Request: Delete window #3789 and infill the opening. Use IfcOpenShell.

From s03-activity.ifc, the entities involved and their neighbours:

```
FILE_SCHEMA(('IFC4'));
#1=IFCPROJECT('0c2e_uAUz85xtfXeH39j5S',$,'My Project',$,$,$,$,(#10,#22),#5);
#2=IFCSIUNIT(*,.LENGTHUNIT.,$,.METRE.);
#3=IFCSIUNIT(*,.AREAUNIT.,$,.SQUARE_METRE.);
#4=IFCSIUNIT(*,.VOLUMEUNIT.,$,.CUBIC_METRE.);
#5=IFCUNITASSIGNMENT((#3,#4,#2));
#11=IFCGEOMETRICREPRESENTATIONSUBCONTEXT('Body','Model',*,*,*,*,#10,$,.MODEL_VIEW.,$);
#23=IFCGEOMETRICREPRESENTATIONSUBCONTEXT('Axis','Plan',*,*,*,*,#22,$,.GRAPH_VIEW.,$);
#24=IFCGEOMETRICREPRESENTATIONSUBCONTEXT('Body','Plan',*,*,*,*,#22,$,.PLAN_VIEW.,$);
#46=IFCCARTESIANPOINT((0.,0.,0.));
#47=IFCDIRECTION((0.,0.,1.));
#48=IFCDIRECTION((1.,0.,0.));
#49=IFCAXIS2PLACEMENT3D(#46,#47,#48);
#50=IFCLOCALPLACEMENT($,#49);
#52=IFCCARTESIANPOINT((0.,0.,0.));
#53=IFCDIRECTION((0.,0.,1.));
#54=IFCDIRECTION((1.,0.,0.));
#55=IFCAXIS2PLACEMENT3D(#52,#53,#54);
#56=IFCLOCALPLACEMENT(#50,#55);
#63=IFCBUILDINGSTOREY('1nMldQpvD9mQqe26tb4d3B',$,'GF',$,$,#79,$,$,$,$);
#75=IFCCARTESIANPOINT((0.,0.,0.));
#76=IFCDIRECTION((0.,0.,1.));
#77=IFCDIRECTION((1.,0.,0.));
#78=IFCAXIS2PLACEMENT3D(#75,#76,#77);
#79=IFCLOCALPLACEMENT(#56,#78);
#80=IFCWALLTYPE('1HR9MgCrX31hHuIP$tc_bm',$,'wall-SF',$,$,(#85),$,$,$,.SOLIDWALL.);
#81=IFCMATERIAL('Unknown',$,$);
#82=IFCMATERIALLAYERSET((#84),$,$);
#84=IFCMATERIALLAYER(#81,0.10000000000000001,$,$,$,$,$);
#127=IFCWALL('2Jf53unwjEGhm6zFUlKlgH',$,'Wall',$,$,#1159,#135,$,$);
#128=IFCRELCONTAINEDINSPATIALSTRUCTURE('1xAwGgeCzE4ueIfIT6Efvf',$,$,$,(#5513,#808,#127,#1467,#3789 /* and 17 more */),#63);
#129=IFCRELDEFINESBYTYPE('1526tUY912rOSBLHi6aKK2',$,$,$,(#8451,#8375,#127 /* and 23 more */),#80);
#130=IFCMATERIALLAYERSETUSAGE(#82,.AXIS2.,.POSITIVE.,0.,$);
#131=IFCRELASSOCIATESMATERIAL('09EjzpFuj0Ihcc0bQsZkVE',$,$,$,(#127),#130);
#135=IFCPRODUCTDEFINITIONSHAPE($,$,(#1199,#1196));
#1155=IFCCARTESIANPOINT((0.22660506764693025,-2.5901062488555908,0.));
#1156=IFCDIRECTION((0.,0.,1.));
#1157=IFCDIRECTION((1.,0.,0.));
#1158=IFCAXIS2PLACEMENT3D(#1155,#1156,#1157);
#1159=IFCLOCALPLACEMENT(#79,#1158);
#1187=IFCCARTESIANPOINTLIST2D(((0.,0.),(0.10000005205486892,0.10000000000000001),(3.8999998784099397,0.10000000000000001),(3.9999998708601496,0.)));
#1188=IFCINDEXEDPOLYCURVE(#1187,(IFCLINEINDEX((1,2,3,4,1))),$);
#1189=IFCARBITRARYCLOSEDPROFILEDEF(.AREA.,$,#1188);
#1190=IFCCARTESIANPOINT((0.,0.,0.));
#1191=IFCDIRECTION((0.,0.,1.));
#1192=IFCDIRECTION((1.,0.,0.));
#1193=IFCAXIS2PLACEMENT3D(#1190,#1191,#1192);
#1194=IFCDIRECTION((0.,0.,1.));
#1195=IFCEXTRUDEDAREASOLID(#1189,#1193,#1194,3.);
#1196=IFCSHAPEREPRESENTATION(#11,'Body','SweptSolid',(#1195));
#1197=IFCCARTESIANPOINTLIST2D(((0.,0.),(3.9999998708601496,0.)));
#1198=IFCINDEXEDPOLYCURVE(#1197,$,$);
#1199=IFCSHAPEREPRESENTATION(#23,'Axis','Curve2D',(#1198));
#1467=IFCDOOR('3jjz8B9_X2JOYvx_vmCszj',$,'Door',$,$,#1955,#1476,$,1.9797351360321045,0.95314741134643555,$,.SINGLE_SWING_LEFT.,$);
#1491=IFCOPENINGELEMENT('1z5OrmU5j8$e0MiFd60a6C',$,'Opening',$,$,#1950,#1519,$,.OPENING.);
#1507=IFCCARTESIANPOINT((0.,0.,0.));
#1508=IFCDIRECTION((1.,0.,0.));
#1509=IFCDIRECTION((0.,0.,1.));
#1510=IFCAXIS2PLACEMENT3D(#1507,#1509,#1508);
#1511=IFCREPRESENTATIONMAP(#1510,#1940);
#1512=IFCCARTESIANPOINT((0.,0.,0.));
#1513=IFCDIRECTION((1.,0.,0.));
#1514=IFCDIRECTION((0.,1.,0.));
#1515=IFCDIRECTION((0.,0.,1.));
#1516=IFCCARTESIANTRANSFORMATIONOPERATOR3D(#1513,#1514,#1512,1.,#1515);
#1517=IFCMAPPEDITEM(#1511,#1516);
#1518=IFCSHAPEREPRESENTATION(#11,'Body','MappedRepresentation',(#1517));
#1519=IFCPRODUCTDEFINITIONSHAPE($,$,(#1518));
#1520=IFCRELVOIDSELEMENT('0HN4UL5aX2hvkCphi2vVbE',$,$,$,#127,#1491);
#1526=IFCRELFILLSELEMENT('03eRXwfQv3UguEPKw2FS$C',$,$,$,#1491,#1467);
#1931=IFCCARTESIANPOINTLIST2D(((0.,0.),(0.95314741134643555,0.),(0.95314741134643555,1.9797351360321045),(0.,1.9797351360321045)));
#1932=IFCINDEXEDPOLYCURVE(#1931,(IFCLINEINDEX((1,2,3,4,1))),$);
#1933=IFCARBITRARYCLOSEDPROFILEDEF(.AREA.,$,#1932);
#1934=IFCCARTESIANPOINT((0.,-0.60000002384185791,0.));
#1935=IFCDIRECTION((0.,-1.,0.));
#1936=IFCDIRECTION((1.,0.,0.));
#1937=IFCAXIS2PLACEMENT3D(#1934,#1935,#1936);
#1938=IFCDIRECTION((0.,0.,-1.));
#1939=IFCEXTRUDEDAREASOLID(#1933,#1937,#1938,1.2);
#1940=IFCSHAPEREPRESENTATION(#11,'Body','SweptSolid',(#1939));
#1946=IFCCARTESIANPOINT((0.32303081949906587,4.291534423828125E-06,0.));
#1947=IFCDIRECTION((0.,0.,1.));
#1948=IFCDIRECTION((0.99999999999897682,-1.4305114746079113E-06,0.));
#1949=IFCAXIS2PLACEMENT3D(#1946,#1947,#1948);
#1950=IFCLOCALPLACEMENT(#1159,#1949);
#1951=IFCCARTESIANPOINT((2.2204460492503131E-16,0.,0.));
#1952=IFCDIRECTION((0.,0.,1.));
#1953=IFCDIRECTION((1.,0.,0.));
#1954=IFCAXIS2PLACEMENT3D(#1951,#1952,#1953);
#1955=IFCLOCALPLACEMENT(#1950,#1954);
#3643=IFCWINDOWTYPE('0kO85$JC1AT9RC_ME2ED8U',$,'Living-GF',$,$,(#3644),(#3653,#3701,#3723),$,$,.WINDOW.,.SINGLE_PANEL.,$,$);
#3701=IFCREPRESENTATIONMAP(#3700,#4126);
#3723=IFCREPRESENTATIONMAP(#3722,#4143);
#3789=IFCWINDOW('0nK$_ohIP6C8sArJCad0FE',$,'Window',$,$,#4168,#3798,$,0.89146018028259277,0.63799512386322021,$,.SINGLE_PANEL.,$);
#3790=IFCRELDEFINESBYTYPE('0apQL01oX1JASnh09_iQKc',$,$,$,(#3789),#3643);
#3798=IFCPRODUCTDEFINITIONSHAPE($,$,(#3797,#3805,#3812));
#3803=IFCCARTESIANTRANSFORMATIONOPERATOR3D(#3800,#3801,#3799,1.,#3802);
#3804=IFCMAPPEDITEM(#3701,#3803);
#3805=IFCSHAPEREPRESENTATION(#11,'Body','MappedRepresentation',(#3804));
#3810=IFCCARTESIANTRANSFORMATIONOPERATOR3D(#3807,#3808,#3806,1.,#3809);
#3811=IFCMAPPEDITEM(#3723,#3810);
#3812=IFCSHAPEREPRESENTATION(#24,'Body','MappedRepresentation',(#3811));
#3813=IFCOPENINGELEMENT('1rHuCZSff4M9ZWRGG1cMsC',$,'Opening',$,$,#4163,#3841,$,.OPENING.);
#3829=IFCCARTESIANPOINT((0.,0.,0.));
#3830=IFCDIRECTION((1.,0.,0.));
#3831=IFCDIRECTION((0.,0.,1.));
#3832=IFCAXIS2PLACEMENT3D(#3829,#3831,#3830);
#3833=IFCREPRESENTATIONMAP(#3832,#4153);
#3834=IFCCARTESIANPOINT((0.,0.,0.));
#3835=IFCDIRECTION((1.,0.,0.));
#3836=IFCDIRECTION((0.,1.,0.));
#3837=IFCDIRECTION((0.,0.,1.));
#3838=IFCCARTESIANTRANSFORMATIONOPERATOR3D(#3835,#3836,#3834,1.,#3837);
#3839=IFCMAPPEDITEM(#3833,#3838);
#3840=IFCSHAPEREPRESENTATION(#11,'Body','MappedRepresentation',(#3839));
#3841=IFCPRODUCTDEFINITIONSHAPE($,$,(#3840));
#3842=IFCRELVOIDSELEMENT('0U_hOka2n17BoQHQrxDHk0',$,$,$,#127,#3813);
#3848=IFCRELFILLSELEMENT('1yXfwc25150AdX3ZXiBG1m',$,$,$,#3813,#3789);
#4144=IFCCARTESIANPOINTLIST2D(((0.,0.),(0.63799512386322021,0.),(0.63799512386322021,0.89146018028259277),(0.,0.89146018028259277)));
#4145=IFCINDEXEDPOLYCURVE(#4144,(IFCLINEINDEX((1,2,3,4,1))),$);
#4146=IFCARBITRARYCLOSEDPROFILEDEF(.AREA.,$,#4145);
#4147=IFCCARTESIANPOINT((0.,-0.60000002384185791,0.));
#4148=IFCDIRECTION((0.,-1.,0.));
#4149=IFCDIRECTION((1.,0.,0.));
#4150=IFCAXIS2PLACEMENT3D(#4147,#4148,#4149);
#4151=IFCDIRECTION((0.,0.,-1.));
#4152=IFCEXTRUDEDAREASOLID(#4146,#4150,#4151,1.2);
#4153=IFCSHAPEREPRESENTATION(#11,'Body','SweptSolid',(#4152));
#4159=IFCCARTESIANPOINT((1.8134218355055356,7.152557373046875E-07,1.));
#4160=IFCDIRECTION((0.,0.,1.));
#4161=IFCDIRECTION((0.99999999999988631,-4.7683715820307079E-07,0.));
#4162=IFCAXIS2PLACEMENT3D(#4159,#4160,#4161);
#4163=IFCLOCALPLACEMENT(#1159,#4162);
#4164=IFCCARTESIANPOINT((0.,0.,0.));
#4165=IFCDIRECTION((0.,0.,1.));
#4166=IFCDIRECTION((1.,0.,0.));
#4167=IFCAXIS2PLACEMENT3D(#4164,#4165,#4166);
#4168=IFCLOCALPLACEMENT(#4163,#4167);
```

```python
import ifcopenshell
import ifcopenshell.api.feature
import ifcopenshell.api.root
import ifcopenshell.geom
import ifcopenshell.util.shape

model = ifcopenshell.open("s03-activity.ifc")
settings = ifcopenshell.geom.settings()


def volume(element):
    """Net volume in cubic metres, openings subtracted."""
    shape = ifcopenshell.geom.create_shape(settings, element)
    return ifcopenshell.util.shape.get_volume(shape.geometry)


window = model.by_guid("0nK$_ohIP6C8sArJCad0FE")
opening = window.FillsVoids[0].RelatingOpeningElement
wall = opening.VoidsElements[0].RelatingBuildingElement
before = volume(wall)

ifcopenshell.api.root.remove_product(model, product=window)
ifcopenshell.api.feature.remove_feature(model, feature=opening)

after = volume(wall)

print(f"wall volume {before:.3f} -> {after:.3f} m3")

model.write("s03-activity_edited.ifc")
```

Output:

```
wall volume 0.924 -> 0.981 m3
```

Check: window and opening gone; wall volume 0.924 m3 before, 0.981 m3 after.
